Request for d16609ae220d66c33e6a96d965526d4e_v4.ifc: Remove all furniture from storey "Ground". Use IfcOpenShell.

First a look at what the model holds.

```python
import ifcopenshell
import ifcopenshell.util.element

model = ifcopenshell.open("d16609ae220d66c33e6a96d965526d4e_v4.ifc")
print(model.schema)
storey = next(s for s in model.by_type("IfcBuildingStorey") if s.Name == "Ground")
furniture = [e for e in ifcopenshell.util.element.get_decomposition(storey) if e.is_a("IfcFurnishingElement")]
seen = {}
for e in furniture:
    element_type = ifcopenshell.util.element.get_type(e)
    name = element_type.Name if element_type not in (None, e) else None
    seen[name] = seen.get(name, 0) + 1
for name, count in sorted(seen.items(), key=str):
    print(count, "x", name)
```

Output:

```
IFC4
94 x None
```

```python
import ifcopenshell
import ifcopenshell.api.root
import ifcopenshell.util.element

model = ifcopenshell.open("d16609ae220d66c33e6a96d965526d4e_v4.ifc")

storey = next(s for s in model.by_type("IfcBuildingStorey") if s.Name == "Ground")
furniture = [e for e in ifcopenshell.util.element.get_decomposition(storey) if e.is_a("IfcFurnishingElement")]

for e in furniture:
    ifcopenshell.api.root.remove_product(model, product=e)
print(len(furniture), "removed")

model.write("d16609ae220d66c33e6a96d965526d4e_v4_v2.ifc")
```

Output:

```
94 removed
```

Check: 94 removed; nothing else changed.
